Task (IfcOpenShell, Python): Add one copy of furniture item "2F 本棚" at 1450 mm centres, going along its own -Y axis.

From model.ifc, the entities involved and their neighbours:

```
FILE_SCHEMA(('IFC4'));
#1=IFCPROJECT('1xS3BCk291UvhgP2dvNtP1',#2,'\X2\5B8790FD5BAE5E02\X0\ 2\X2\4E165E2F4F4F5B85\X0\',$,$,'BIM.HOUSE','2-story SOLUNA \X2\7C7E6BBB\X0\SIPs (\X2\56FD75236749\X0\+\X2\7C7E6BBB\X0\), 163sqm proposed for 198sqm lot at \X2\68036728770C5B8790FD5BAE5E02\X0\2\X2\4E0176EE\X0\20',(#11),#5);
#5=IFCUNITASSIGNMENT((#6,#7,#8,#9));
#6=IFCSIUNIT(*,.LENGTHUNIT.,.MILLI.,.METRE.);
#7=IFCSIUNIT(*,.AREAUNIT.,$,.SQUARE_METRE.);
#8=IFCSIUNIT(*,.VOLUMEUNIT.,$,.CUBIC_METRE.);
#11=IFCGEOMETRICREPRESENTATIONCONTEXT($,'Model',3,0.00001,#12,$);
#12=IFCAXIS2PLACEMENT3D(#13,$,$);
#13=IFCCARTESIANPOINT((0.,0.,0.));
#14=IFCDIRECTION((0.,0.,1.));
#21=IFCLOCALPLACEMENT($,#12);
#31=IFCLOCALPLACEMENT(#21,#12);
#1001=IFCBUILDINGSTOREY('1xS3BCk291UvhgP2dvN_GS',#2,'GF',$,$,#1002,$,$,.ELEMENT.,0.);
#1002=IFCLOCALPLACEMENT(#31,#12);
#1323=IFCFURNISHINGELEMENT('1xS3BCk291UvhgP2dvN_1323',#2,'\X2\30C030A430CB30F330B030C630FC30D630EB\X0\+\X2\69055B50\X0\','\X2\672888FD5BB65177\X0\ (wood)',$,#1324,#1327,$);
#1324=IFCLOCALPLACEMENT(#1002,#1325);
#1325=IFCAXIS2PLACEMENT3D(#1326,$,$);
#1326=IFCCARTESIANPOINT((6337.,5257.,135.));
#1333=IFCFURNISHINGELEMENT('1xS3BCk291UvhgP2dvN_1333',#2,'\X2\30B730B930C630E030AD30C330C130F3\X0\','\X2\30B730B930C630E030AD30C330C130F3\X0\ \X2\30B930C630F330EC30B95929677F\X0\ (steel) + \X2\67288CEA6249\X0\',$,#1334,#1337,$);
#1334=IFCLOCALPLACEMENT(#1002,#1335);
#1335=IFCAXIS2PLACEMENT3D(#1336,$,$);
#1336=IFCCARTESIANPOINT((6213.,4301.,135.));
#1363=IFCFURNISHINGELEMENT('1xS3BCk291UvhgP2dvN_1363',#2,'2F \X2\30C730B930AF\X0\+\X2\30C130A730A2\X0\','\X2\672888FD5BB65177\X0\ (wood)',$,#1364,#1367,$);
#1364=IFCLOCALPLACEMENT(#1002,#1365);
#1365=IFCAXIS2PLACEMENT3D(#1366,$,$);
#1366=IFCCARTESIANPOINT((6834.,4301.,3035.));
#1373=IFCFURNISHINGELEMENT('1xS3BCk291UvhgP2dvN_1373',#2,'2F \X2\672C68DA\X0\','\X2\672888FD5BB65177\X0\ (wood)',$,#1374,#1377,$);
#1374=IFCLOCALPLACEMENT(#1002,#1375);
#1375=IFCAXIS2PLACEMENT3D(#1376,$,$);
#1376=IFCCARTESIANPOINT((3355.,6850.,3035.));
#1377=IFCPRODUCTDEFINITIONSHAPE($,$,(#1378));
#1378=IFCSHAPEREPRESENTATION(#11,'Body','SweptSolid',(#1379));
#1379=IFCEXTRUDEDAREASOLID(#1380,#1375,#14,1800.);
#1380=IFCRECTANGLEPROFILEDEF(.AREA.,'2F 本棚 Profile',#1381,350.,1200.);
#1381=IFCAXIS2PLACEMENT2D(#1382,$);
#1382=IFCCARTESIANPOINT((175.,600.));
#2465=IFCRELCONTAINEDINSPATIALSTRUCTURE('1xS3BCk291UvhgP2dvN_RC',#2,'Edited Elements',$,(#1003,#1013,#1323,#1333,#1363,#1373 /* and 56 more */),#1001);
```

```python
import ifcopenshell
import ifcopenshell.api.geometry
import ifcopenshell.api.root
import ifcopenshell.util.element
import ifcopenshell.util.placement

model = ifcopenshell.open("model.ifc")


def reuse_history(source, copy):
    """copy_class also copies each property set's owner history, people and application; keep the originals."""
    for rel in copy.IsDefinedBy:
        if rel.is_a("IfcRelDefinesByProperties") and (history := rel.RelatingPropertyDefinition.OwnerHistory):
            rel.RelatingPropertyDefinition.OwnerHistory = source.OwnerHistory
            ifcopenshell.util.element.remove_deep2(model, history)


source = model.by_guid("1xS3BCk291UvhgP2dvN_1373")
base = ifcopenshell.util.placement.get_local_placement(source.ObjectPlacement)
step = -base[:3, 1] * 1450.0

for i in range(1, 2):
    copy = ifcopenshell.api.root.copy_class(model, product=source)
    copy.Representation = ifcopenshell.util.element.copy_deep(
        model, source.Representation, exclude=["IfcGeometricRepresentationContext", "IfcRepresentationMap"]
    )
    reuse_history(source, copy)
    matrix = base.copy()
    matrix[:3, 3] += i * step
    print("added at", matrix[:3, 3].round(3) + 0.0)
    ifcopenshell.api.geometry.edit_object_placement(model, product=copy, matrix=matrix, is_si=False)

model.write("model_updated.ifc")
```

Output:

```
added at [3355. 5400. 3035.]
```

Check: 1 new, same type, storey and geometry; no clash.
